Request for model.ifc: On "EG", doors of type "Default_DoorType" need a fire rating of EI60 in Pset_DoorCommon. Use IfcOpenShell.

First a look at what the model holds.

```python
import ifcopenshell
import ifcopenshell.util.element

model = ifcopenshell.open("model.ifc")
print(model.schema)
storey = next(s for s in model.by_type("IfcBuildingStorey") if s.Name == "EG")
doors = [e for e in ifcopenshell.util.element.get_decomposition(storey) if e.is_a("IfcDoor")]
seen = {}
for e in doors:
    element_type = ifcopenshell.util.element.get_type(e)
    key = (element_type.Name if element_type != e and element_type else None, ifcopenshell.util.element.get_pset(e, "Pset_DoorCommon", "FireRating"))
    seen[key] = seen.get(key, 0) + 1
for (name, value), count in sorted(seen.items(), key=str):
    print(count, "x", name, "|", value)
```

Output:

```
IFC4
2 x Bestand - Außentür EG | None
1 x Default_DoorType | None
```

```python
import ifcopenshell
import ifcopenshell.api.pset
import ifcopenshell.util.element

model = ifcopenshell.open("model.ifc")

storey = next(s for s in model.by_type("IfcBuildingStorey") if s.Name == "EG")
doors = [e for e in ifcopenshell.util.element.get_decomposition(storey) if e.is_a("IfcDoor")]

count = 0
for e in doors:
    element_type = ifcopenshell.util.element.get_type(e)
    if element_type in (None, e) or element_type.Name != "Default_DoorType":
        continue
    # add_pset returns the element's existing set when there is one.
    pset = ifcopenshell.api.pset.add_pset(model, product=e, name="Pset_DoorCommon")
    ifcopenshell.api.pset.edit_pset(model, pset=pset, properties={"FireRating": "EI60"})
    count += 1

print(count, "doors updated")

model.write("model_edited.ifc")
```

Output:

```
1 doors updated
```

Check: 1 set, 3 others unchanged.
